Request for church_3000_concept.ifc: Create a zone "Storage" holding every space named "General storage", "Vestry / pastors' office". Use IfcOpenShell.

First a look at what the model holds.

```python
import ifcopenshell

model = ifcopenshell.open("church_3000_concept.ifc")
print(model.schema)
seen = {}
for space in model.by_type("IfcSpace"):
    seen[space.LongName] = seen.get(space.LongName, 0) + 1
for name, count in sorted(seen.items(), key=str):
    print(count, "x", name)
print("zones:", [z.Name for z in model.by_type("IfcZone")][:20])
```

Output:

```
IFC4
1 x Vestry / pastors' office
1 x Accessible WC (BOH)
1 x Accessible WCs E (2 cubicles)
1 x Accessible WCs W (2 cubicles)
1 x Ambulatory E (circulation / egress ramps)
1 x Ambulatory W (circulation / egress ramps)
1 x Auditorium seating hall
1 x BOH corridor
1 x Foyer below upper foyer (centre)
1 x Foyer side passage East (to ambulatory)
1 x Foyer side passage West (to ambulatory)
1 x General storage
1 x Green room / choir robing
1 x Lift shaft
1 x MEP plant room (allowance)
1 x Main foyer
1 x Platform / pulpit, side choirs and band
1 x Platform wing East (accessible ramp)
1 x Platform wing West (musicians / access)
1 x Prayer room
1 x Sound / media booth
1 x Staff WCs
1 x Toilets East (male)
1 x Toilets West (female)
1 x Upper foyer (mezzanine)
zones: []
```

```python
import ifcopenshell
import ifcopenshell.api.group
import ifcopenshell.api.root

model = ifcopenshell.open("church_3000_concept.ifc")

names = {"General storage", "Vestry / pastors' office"}
spaces = [s for s in model.by_type("IfcSpace") if s.LongName in names]

zone = ifcopenshell.api.root.create_entity(model, ifc_class="IfcZone", name="Storage")
ifcopenshell.api.group.assign_group(model, products=spaces, group=zone)
print(len(spaces), "spaces in", zone.Name)

model.write("church_3000_concept-out.ifc")
```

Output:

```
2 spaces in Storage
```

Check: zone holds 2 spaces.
